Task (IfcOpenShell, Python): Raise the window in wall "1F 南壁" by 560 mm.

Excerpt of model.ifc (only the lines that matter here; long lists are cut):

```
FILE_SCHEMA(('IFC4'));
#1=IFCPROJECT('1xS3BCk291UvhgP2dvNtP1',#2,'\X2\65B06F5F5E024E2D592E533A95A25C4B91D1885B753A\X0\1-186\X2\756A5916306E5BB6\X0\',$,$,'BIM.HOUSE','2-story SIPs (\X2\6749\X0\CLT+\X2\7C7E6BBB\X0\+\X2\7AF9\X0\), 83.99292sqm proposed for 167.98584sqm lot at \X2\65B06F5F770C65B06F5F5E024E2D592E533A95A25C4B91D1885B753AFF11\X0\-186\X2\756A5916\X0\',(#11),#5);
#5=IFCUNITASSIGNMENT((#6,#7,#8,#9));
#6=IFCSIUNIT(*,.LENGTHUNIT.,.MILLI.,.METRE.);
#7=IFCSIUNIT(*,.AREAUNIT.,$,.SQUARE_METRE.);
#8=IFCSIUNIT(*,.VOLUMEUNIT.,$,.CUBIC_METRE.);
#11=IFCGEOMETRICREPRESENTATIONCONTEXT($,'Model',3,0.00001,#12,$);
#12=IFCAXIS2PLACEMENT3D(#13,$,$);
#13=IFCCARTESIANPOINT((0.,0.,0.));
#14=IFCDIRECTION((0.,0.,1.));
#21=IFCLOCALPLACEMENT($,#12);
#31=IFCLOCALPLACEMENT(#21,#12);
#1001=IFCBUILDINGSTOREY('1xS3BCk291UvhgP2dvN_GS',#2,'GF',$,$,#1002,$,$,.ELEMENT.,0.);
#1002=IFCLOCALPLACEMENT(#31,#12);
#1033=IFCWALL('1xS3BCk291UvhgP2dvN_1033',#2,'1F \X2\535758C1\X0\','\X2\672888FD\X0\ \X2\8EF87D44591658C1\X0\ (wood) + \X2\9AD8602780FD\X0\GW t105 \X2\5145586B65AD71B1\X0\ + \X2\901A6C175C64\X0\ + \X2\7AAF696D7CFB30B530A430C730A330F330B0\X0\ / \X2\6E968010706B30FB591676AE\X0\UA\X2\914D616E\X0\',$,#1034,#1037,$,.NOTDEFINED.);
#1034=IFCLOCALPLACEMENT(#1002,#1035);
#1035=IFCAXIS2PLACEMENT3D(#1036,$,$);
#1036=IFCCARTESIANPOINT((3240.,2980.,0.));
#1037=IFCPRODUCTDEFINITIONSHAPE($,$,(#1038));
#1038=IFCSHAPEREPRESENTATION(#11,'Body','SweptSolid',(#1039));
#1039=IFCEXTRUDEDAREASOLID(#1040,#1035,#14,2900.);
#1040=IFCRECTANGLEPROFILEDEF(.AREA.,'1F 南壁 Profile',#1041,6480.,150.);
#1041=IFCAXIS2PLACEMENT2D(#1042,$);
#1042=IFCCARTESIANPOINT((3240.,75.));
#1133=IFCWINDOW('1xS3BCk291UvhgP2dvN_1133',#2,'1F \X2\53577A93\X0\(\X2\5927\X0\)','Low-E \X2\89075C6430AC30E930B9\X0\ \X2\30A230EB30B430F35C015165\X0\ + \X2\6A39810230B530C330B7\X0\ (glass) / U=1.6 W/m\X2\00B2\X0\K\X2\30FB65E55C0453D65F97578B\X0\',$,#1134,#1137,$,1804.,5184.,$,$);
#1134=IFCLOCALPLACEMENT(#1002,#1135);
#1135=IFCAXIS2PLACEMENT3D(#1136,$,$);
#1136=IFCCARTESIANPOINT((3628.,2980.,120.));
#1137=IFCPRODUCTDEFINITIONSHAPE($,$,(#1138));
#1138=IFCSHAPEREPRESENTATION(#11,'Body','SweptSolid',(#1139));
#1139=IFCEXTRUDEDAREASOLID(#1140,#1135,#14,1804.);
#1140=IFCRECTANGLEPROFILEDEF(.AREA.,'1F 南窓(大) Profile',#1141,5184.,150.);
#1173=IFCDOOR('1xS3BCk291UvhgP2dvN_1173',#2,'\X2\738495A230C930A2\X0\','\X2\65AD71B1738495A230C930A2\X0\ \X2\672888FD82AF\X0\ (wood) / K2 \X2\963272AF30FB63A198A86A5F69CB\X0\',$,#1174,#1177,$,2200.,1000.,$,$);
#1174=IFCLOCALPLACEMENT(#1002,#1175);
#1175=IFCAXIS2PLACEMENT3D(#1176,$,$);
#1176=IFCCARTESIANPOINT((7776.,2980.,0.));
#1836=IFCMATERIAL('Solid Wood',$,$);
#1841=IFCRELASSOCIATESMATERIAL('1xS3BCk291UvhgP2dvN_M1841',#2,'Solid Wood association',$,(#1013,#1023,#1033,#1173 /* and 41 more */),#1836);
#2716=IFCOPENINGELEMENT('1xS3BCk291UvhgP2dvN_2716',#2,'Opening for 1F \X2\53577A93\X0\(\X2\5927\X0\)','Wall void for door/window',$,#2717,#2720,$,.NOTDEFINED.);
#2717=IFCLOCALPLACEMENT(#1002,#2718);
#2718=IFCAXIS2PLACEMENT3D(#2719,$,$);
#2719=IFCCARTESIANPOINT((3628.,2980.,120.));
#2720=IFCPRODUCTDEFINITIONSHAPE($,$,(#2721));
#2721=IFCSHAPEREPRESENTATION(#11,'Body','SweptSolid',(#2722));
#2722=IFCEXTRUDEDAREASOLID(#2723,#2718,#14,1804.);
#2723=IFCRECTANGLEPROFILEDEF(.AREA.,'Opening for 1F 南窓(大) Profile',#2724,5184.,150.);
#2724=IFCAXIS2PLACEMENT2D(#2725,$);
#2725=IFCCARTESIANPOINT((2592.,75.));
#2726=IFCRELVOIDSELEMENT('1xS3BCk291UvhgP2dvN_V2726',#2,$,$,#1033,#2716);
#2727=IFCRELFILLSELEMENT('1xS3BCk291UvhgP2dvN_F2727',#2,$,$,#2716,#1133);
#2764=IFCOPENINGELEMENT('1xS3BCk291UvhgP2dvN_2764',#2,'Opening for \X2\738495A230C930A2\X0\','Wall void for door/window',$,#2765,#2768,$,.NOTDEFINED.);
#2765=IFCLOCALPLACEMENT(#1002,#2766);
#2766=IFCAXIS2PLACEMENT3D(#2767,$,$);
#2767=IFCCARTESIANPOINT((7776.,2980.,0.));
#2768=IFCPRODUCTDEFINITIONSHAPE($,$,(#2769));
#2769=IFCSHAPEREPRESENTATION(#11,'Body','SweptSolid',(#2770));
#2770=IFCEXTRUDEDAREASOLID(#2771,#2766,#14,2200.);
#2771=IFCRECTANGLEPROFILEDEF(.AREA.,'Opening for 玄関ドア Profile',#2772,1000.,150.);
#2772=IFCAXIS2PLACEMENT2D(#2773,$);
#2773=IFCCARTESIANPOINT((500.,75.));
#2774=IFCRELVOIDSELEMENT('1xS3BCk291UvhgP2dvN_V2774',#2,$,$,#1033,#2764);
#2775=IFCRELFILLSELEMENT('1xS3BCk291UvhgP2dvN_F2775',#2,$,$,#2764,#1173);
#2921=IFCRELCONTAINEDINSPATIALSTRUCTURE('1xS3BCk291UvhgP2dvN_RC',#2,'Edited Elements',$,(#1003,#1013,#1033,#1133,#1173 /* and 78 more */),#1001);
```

```python
import numpy as np
import ifcopenshell
import ifcopenshell.api.geometry
import ifcopenshell.util.placement
import ifcopenshell.util.unit

model = ifcopenshell.open("model.ifc")
unit_scale = ifcopenshell.util.unit.calculate_unit_scale(model)

window = model.by_id(1133)
opening = window.FillsVoids[0].RelatingOpeningElement
dz = 560.0

shift = np.array([0.0, 0.0, dz])
# The window is not placed relative to its opening, so move both.
for product in (opening, window):
    matrix = ifcopenshell.util.placement.get_local_placement(product.ObjectPlacement)
    matrix[:3, 3] += shift
    ifcopenshell.api.geometry.edit_object_placement(model, product=product, matrix=matrix, is_si=False)

print(f"moved by {dz * unit_scale:+.3f} m")

model.write("model_rev.ifc")
```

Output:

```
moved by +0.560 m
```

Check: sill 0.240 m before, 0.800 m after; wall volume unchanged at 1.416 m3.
